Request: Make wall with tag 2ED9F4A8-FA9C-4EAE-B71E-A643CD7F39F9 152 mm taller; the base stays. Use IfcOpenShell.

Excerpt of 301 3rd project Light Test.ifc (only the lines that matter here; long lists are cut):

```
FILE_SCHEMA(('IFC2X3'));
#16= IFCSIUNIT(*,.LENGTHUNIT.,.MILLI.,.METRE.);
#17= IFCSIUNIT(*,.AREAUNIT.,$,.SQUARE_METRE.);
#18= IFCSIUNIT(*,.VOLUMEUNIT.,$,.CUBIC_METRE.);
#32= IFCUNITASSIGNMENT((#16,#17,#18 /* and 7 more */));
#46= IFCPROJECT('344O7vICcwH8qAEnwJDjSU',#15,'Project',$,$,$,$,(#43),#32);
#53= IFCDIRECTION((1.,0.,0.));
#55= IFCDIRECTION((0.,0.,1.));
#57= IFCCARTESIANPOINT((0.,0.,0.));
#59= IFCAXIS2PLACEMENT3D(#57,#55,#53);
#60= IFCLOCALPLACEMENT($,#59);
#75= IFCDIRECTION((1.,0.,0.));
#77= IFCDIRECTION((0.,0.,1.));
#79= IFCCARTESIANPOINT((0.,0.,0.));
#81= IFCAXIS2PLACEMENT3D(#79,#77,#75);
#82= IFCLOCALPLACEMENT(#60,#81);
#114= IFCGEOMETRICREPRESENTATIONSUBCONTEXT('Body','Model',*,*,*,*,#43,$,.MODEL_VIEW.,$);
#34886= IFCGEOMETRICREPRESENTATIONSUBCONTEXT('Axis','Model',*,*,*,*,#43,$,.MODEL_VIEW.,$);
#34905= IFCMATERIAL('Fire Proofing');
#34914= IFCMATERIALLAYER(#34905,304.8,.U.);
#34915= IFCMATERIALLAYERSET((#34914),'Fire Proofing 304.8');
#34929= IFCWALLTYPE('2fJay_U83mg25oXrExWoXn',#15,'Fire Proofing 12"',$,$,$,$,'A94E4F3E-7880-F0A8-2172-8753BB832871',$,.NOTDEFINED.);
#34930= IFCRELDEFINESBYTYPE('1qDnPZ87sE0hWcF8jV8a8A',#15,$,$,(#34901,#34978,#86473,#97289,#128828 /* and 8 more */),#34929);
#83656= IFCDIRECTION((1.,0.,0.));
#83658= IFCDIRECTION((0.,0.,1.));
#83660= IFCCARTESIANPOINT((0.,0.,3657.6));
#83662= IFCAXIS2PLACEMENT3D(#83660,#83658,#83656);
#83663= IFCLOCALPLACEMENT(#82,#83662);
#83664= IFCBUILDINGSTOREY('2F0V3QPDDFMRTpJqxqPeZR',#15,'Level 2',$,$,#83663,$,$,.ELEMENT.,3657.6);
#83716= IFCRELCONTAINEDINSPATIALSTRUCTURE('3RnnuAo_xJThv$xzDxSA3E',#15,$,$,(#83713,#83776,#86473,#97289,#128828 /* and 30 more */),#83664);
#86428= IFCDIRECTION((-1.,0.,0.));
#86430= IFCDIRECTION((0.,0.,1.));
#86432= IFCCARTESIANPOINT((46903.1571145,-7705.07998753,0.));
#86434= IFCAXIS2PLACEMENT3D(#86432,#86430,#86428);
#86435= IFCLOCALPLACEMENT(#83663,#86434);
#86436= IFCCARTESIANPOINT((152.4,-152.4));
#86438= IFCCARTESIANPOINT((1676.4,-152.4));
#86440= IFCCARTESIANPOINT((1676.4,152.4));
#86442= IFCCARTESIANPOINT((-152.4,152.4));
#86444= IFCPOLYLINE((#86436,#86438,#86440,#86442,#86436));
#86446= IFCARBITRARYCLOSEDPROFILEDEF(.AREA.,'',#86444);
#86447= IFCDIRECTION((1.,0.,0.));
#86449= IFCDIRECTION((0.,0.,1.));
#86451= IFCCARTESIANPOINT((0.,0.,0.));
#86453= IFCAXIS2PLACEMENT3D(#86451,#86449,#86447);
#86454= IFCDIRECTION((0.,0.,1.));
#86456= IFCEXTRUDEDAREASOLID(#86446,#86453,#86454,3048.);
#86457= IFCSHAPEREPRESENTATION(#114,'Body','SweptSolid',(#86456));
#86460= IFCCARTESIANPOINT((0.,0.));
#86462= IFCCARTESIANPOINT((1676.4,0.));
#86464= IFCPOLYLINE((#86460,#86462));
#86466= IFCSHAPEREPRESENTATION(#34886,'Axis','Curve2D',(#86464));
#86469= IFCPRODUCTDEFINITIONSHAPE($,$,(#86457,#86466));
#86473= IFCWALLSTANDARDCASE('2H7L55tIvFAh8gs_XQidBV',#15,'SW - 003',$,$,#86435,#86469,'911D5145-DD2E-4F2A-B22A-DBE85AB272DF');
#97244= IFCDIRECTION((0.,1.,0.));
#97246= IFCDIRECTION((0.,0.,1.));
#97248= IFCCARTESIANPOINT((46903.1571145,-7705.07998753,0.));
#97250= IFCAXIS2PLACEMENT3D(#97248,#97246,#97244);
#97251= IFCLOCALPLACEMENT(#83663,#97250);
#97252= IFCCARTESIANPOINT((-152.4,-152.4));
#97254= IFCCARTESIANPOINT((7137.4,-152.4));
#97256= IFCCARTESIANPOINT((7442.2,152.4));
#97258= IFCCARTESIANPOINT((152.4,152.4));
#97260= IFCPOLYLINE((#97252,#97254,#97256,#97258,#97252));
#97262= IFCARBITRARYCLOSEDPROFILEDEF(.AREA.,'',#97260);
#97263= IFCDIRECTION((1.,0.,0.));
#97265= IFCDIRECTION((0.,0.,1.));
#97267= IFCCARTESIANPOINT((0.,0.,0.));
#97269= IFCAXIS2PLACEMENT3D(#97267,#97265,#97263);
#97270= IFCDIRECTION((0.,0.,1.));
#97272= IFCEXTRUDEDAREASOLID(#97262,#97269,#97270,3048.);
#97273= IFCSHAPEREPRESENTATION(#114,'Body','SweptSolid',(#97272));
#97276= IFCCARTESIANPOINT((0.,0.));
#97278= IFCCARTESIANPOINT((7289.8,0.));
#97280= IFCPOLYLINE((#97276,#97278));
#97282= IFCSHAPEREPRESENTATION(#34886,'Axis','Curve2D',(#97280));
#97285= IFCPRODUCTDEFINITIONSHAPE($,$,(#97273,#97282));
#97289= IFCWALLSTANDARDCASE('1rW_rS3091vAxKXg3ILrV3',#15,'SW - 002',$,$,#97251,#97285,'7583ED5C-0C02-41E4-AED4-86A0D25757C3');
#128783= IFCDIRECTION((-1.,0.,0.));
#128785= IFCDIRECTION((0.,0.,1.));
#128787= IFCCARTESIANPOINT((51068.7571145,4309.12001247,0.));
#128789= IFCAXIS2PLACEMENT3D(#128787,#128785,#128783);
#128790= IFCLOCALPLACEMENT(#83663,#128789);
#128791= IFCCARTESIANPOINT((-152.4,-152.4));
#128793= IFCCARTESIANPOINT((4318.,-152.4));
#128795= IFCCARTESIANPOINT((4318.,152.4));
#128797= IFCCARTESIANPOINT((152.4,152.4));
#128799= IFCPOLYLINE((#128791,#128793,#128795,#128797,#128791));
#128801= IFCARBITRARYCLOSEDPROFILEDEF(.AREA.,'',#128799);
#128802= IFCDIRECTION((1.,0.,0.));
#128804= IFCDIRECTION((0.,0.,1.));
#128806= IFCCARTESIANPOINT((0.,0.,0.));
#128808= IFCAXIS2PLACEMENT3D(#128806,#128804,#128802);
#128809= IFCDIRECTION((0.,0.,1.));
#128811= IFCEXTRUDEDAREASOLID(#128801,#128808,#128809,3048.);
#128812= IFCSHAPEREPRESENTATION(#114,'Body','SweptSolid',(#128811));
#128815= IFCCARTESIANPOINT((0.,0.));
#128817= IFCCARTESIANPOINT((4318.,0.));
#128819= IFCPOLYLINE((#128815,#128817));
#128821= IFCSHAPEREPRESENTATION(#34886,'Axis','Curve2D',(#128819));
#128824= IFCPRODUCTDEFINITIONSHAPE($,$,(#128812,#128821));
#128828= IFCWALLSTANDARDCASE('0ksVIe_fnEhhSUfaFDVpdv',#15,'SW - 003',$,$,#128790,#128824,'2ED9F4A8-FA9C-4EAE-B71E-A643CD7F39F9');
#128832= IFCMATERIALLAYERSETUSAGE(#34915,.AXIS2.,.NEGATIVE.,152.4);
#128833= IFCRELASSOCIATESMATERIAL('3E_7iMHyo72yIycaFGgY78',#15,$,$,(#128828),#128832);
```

```python
import ifcopenshell
import ifcopenshell.geom
import ifcopenshell.util.representation
import ifcopenshell.util.shape
import ifcopenshell.util.unit

model = ifcopenshell.open("301 3rd project Light Test.ifc")
unit_scale = ifcopenshell.util.unit.calculate_unit_scale(model)
settings = ifcopenshell.geom.settings()


def volume(element):
    """Net volume in cubic metres, openings subtracted."""
    shape = ifcopenshell.geom.create_shape(settings, element)
    return ifcopenshell.util.shape.get_volume(shape.geometry)


wall = model.by_guid("0ksVIe_fnEhhSUfaFDVpdv")
before = volume(wall)

body = ifcopenshell.util.representation.get_representation(wall, "Model", "Body")
solid = body.Items[0]
old_height = solid.Depth
solid.Depth += 0.152 / unit_scale
after = volume(wall)

print(f"height {old_height:g} -> {solid.Depth:g}, volume {before:.3f} -> {after:.3f} m3")

model.write("301 3rd project Light Test_v2.ifc")
```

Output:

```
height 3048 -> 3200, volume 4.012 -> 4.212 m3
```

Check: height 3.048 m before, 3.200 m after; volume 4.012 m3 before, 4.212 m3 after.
